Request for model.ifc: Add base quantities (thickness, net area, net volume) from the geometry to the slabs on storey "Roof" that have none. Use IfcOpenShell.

First a look at what the model holds.

```python
import ifcopenshell
import ifcopenshell.util.element
import ifcopenshell.util.unit

model = ifcopenshell.open("model.ifc")
print(model.schema)
for unit_type in ("LENGTHUNIT", "AREAUNIT", "VOLUMEUNIT"):
    print(unit_type, ifcopenshell.util.unit.calculate_unit_scale(model, unit_type))
storey = next(s for s in model.by_type("IfcBuildingStorey") if s.Name == "Roof")
slabs = [e for e in ifcopenshell.util.element.get_decomposition(storey) if e.is_a("IfcSlab")]
for e in sorted(slabs, key=lambda e: e.id()):
    print(e.id(), e.is_a(), e.Name, list(ifcopenshell.util.element.get_psets(e, qtos_only=True)), sep=" | ")
```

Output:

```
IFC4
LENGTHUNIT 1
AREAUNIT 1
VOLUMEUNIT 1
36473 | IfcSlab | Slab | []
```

```python
import ifcopenshell
import ifcopenshell.api.pset
import ifcopenshell.geom
import ifcopenshell.util.element
import ifcopenshell.util.shape
import ifcopenshell.util.unit

model = ifcopenshell.open("model.ifc")
unit_scale = ifcopenshell.util.unit.calculate_unit_scale(model)
area_scale = ifcopenshell.util.unit.calculate_unit_scale(model, "AREAUNIT")
volume_scale = ifcopenshell.util.unit.calculate_unit_scale(model, "VOLUMEUNIT")
settings = ifcopenshell.geom.settings()

storey = next(s for s in model.by_type("IfcBuildingStorey") if s.Name == "Roof")
slabs = [e for e in ifcopenshell.util.element.get_decomposition(storey) if e.is_a("IfcSlab")]

for e in sorted(slabs, key=lambda e: e.id()):
    if ifcopenshell.util.element.get_psets(e, qtos_only=True, should_inherit=False):
        continue
    # Geometry comes back in metres, in the element's own axes.
    shape = ifcopenshell.geom.create_shape(settings, e)
    values = {
        "Width": ifcopenshell.util.shape.get_z(shape.geometry) / unit_scale,
        "NetArea": ifcopenshell.util.shape.get_footprint_area(shape.geometry) / area_scale,
        "NetVolume": ifcopenshell.util.shape.get_volume(shape.geometry) / volume_scale,
    }
    qto = ifcopenshell.api.pset.add_qto(model, product=e, name="Qto_SlabBaseQuantities")
    ifcopenshell.api.pset.edit_qto(model, qto=qto, properties=values)
    print(e.id(), {k: round(v, 3) for k, v in values.items()})

model.write("model_edited.ifc")
```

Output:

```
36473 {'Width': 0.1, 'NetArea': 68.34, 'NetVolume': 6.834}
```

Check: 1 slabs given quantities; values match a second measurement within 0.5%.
